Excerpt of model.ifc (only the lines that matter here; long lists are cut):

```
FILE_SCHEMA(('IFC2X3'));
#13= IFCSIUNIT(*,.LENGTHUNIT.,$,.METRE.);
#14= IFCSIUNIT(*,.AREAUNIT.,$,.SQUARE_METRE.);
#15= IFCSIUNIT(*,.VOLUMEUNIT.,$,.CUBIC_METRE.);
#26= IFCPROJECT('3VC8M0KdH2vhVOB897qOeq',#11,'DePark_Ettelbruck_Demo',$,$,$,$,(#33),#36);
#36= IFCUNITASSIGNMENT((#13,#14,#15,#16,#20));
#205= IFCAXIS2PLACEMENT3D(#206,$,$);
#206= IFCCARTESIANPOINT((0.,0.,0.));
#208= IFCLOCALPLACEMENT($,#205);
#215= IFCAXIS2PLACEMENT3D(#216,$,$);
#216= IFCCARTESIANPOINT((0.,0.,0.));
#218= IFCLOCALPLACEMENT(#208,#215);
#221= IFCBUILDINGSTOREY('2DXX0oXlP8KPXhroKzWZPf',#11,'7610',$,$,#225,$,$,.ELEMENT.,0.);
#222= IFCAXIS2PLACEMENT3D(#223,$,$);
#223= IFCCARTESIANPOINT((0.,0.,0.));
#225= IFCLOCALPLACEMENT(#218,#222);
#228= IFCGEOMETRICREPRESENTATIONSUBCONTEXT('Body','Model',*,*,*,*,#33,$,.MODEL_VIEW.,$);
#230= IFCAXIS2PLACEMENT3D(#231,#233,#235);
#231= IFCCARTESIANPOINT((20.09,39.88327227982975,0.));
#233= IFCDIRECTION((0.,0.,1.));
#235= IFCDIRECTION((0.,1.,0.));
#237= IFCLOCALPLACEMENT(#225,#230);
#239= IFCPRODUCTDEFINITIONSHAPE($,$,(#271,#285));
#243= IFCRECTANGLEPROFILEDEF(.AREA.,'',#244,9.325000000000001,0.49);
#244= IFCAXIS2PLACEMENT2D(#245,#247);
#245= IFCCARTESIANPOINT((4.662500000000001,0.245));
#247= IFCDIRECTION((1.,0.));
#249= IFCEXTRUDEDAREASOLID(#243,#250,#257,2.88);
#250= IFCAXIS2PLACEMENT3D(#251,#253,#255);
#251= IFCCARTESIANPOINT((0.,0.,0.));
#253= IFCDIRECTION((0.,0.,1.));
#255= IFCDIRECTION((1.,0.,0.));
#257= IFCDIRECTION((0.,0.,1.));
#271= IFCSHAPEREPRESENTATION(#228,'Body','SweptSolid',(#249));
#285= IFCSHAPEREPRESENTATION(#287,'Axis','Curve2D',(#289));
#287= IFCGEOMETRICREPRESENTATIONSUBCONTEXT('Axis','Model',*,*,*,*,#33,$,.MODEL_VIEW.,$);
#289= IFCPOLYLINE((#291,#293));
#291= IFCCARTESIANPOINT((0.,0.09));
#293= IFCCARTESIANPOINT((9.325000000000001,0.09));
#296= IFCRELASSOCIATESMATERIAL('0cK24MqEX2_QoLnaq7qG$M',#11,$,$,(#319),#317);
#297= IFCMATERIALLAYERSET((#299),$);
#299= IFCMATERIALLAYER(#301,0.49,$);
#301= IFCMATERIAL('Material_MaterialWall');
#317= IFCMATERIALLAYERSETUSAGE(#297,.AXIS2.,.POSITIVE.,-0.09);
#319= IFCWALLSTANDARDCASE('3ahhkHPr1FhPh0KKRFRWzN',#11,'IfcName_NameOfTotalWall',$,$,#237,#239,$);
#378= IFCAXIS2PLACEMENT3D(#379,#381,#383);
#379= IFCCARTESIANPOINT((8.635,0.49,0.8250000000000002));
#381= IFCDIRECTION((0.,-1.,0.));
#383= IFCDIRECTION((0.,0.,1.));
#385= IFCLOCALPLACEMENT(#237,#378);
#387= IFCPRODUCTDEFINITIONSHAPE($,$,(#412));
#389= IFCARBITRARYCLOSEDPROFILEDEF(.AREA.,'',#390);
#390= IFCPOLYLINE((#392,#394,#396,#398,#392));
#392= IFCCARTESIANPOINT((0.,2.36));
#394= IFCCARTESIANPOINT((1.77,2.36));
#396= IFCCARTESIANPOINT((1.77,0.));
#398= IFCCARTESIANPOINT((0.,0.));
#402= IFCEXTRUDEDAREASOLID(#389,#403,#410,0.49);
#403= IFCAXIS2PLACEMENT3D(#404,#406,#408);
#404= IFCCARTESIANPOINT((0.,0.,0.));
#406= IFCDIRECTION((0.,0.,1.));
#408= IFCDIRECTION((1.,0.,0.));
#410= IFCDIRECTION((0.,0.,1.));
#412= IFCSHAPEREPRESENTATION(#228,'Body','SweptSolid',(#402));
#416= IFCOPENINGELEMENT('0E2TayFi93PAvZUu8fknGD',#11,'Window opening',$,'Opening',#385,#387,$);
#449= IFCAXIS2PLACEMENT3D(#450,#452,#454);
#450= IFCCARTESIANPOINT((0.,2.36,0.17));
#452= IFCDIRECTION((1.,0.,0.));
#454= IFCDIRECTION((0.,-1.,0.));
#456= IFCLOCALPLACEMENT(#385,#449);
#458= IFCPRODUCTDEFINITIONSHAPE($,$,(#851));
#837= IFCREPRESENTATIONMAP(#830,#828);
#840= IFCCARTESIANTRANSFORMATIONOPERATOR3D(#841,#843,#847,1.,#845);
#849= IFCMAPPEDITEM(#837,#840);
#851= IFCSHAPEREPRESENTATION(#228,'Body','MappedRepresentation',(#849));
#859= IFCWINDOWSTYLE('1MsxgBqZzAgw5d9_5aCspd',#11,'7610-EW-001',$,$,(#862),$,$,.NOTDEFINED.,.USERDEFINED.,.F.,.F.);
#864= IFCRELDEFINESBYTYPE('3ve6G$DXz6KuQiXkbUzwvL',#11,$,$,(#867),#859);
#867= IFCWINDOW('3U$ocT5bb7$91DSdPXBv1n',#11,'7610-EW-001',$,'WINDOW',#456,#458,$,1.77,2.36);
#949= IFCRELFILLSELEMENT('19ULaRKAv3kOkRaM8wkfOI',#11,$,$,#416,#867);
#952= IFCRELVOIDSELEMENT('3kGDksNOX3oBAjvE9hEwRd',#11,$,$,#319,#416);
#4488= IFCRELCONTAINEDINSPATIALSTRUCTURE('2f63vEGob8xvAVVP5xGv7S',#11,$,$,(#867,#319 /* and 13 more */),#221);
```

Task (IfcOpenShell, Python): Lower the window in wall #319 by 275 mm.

```python
import numpy as np
import ifcopenshell
import ifcopenshell.api.geometry
import ifcopenshell.util.placement
import ifcopenshell.util.unit

model = ifcopenshell.open("model.ifc")
unit_scale = ifcopenshell.util.unit.calculate_unit_scale(model)

window = model.by_guid("3U$ocT5bb7$91DSdPXBv1n")
opening = window.FillsVoids[0].RelatingOpeningElement
dz = -0.275

shift = np.array([0.0, 0.0, dz])
# The window is placed relative to its opening, so it follows when the opening moves.
matrix = ifcopenshell.util.placement.get_local_placement(opening.ObjectPlacement)
matrix[:3, 3] += shift
ifcopenshell.api.geometry.edit_object_placement(
    model, product=opening, matrix=matrix, is_si=False, should_transform_children=True
)

print(f"moved by {dz * unit_scale:+.3f} m")

model.write("model_edited.ifc")
```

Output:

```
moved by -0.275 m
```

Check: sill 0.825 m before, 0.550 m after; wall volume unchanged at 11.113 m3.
